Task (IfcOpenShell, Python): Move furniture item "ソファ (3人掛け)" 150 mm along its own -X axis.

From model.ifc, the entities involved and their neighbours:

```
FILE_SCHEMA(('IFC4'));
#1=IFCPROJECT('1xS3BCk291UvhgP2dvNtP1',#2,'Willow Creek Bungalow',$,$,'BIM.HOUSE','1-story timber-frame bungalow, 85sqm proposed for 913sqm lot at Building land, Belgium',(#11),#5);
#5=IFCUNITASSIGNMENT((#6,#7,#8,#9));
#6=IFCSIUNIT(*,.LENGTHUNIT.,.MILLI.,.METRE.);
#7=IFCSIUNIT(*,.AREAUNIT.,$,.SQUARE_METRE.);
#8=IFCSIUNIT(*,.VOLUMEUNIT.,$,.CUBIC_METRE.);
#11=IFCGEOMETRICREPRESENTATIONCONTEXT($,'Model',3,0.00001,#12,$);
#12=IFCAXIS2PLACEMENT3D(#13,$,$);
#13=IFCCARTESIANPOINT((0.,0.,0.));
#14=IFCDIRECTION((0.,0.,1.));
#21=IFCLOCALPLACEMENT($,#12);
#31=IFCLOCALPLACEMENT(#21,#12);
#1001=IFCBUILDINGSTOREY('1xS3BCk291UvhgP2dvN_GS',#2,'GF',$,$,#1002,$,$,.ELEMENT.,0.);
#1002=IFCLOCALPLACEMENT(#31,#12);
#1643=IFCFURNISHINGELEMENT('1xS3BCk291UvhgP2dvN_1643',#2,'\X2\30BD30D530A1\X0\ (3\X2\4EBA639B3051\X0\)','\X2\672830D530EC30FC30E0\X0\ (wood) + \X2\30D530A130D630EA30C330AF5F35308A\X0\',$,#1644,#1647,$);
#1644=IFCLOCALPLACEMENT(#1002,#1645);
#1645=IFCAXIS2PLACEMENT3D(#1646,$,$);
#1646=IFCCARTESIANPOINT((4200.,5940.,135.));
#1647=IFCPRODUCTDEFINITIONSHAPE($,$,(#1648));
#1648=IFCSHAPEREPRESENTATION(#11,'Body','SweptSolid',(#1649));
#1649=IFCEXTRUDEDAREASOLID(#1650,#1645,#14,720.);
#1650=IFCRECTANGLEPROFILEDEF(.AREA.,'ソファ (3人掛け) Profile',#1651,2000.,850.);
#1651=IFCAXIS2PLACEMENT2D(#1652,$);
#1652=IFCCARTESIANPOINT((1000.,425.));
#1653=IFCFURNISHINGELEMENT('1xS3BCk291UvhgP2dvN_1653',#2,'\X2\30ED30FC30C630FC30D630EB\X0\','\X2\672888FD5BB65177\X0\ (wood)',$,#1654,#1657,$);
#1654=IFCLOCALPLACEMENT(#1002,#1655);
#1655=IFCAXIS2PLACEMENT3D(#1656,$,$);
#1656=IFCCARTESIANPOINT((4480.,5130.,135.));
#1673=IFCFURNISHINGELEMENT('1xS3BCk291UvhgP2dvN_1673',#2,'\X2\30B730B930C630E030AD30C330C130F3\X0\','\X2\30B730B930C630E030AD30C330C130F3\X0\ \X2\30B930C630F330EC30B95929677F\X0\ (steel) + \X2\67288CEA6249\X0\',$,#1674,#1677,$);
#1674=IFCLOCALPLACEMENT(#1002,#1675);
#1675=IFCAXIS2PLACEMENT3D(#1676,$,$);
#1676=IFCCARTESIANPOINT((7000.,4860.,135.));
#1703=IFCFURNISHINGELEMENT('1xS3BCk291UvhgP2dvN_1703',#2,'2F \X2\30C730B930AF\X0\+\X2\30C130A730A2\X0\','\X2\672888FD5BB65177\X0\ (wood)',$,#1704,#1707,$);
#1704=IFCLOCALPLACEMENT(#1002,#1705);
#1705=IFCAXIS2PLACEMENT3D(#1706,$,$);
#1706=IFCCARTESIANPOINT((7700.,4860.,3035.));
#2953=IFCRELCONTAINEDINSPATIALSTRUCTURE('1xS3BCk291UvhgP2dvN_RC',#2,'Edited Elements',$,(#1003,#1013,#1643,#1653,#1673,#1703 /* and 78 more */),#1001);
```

```python
import ifcopenshell
import ifcopenshell.api.geometry
import ifcopenshell.util.placement
import ifcopenshell.util.unit

model = ifcopenshell.open("model.ifc")
unit_scale = ifcopenshell.util.unit.calculate_unit_scale(model)

item = model.by_guid("1xS3BCk291UvhgP2dvN_1643")
matrix = ifcopenshell.util.placement.get_local_placement(item.ObjectPlacement)
matrix[:3, 3] -= matrix[:3, 0] * 0.15 / unit_scale
ifcopenshell.api.geometry.edit_object_placement(model, product=item, matrix=matrix, is_si=False)

print(ifcopenshell.util.placement.get_local_placement(item.ObjectPlacement).round(3) + 0.0)

model.write("model-out.ifc")
```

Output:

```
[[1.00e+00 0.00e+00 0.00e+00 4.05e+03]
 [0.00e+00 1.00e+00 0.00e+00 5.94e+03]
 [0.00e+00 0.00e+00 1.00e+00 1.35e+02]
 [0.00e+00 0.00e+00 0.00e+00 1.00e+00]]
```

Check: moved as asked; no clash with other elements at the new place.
